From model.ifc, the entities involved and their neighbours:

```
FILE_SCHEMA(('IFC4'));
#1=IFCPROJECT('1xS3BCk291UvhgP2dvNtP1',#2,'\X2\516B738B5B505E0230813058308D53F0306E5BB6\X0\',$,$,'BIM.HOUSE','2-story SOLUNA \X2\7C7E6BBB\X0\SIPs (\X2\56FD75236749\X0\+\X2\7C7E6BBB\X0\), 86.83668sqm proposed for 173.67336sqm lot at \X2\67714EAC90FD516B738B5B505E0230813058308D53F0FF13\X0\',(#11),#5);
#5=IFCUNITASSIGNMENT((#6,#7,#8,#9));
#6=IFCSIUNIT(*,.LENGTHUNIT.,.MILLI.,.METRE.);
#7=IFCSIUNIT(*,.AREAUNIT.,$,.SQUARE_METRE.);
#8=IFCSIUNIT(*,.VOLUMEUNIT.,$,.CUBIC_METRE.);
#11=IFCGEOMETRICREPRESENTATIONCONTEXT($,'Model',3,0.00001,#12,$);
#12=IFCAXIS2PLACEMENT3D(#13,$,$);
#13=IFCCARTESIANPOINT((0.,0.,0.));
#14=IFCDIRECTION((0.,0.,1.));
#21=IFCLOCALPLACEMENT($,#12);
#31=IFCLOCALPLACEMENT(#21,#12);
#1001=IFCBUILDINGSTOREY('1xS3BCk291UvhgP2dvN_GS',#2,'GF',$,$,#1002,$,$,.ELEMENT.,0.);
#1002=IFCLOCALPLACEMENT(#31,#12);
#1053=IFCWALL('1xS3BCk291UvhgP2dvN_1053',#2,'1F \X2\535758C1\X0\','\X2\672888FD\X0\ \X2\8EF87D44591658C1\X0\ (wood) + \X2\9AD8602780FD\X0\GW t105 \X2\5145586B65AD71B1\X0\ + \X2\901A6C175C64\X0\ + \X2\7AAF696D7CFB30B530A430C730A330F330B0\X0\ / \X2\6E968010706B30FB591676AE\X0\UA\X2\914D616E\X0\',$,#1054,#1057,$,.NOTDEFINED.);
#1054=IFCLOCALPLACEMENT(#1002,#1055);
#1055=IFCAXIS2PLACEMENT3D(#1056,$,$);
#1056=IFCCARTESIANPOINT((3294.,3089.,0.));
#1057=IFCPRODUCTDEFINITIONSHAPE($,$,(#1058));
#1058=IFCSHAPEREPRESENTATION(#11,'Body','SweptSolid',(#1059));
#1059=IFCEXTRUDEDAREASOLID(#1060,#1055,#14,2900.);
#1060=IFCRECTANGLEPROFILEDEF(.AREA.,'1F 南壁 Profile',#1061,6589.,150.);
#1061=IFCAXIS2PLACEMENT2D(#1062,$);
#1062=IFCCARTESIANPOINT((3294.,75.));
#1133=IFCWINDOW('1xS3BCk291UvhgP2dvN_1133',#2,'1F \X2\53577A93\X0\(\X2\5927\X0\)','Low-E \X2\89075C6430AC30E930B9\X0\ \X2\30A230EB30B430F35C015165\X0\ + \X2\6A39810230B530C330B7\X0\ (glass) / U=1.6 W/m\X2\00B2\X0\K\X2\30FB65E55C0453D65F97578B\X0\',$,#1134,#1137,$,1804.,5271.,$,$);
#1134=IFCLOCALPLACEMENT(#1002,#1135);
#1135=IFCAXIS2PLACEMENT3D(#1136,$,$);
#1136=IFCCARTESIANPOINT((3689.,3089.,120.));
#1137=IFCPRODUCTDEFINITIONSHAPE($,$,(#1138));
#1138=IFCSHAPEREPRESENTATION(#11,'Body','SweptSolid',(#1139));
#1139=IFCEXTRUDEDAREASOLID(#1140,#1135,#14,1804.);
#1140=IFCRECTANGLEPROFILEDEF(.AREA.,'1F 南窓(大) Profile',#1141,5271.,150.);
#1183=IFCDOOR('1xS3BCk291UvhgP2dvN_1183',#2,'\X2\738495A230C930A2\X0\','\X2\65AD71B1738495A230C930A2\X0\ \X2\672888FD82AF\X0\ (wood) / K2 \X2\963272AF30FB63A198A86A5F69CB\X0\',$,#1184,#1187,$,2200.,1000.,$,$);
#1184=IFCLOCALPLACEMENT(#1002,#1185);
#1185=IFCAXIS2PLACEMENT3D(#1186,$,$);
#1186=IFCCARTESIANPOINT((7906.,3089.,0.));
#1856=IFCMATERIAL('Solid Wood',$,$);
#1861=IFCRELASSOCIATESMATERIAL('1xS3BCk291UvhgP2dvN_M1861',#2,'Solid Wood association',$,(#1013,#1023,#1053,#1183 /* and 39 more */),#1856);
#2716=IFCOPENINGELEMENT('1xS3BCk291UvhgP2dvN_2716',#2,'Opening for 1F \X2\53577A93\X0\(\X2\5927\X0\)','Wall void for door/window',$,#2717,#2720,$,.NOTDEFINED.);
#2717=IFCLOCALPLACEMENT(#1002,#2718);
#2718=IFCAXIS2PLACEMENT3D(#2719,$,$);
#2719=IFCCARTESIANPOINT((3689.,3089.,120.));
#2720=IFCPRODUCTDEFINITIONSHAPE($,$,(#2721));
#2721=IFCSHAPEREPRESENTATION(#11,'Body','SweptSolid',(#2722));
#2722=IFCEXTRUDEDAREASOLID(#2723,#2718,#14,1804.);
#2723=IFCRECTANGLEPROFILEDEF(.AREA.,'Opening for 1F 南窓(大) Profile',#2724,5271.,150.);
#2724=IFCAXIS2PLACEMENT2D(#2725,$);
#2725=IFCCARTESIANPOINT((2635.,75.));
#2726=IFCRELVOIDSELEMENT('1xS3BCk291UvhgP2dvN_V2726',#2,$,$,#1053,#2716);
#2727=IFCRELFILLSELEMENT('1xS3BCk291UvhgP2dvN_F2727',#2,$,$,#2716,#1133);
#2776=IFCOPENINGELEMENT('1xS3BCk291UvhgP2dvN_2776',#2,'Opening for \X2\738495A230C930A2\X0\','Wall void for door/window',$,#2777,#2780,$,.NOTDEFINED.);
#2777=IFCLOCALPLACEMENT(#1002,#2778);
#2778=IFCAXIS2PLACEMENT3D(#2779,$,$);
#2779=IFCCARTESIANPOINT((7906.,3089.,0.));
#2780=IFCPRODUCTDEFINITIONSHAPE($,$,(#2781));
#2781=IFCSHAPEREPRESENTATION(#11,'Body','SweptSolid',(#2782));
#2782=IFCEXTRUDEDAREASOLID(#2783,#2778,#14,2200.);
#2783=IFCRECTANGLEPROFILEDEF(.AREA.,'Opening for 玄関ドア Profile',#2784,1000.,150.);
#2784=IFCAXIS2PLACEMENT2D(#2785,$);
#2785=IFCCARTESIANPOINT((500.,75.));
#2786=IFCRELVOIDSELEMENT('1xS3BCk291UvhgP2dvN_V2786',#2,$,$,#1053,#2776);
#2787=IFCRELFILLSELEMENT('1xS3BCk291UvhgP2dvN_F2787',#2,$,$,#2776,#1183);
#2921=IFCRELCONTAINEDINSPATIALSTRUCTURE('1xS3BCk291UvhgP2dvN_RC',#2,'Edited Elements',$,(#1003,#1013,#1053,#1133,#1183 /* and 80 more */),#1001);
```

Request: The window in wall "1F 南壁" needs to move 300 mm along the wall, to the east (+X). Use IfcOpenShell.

```python
import ifcopenshell
import ifcopenshell.api.geometry
import ifcopenshell.util.placement

model = ifcopenshell.open("model.ifc")

window = model.by_id(1133)
opening = window.FillsVoids[0].RelatingOpeningElement
wall = opening.VoidsElements[0].RelatingBuildingElement

wall_matrix = ifcopenshell.util.placement.get_local_placement(wall.ObjectPlacement)
shift = wall_matrix[:3, 0] * 300.0
before = ifcopenshell.util.placement.get_local_placement(window.ObjectPlacement)[:3, 3].copy()

# The window is not placed relative to its opening, so move both.
for product in (opening, window):
    matrix = ifcopenshell.util.placement.get_local_placement(product.ObjectPlacement)
    matrix[:3, 3] += shift
    ifcopenshell.api.geometry.edit_object_placement(model, product=product, matrix=matrix, is_si=False)

after = ifcopenshell.util.placement.get_local_placement(window.ObjectPlacement)[:3, 3]
print("window moved by", (after - before).round(3) + 0.0)

model.write("model_updated.ifc")
```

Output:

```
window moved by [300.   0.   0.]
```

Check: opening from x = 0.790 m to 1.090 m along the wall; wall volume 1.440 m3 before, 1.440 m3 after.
